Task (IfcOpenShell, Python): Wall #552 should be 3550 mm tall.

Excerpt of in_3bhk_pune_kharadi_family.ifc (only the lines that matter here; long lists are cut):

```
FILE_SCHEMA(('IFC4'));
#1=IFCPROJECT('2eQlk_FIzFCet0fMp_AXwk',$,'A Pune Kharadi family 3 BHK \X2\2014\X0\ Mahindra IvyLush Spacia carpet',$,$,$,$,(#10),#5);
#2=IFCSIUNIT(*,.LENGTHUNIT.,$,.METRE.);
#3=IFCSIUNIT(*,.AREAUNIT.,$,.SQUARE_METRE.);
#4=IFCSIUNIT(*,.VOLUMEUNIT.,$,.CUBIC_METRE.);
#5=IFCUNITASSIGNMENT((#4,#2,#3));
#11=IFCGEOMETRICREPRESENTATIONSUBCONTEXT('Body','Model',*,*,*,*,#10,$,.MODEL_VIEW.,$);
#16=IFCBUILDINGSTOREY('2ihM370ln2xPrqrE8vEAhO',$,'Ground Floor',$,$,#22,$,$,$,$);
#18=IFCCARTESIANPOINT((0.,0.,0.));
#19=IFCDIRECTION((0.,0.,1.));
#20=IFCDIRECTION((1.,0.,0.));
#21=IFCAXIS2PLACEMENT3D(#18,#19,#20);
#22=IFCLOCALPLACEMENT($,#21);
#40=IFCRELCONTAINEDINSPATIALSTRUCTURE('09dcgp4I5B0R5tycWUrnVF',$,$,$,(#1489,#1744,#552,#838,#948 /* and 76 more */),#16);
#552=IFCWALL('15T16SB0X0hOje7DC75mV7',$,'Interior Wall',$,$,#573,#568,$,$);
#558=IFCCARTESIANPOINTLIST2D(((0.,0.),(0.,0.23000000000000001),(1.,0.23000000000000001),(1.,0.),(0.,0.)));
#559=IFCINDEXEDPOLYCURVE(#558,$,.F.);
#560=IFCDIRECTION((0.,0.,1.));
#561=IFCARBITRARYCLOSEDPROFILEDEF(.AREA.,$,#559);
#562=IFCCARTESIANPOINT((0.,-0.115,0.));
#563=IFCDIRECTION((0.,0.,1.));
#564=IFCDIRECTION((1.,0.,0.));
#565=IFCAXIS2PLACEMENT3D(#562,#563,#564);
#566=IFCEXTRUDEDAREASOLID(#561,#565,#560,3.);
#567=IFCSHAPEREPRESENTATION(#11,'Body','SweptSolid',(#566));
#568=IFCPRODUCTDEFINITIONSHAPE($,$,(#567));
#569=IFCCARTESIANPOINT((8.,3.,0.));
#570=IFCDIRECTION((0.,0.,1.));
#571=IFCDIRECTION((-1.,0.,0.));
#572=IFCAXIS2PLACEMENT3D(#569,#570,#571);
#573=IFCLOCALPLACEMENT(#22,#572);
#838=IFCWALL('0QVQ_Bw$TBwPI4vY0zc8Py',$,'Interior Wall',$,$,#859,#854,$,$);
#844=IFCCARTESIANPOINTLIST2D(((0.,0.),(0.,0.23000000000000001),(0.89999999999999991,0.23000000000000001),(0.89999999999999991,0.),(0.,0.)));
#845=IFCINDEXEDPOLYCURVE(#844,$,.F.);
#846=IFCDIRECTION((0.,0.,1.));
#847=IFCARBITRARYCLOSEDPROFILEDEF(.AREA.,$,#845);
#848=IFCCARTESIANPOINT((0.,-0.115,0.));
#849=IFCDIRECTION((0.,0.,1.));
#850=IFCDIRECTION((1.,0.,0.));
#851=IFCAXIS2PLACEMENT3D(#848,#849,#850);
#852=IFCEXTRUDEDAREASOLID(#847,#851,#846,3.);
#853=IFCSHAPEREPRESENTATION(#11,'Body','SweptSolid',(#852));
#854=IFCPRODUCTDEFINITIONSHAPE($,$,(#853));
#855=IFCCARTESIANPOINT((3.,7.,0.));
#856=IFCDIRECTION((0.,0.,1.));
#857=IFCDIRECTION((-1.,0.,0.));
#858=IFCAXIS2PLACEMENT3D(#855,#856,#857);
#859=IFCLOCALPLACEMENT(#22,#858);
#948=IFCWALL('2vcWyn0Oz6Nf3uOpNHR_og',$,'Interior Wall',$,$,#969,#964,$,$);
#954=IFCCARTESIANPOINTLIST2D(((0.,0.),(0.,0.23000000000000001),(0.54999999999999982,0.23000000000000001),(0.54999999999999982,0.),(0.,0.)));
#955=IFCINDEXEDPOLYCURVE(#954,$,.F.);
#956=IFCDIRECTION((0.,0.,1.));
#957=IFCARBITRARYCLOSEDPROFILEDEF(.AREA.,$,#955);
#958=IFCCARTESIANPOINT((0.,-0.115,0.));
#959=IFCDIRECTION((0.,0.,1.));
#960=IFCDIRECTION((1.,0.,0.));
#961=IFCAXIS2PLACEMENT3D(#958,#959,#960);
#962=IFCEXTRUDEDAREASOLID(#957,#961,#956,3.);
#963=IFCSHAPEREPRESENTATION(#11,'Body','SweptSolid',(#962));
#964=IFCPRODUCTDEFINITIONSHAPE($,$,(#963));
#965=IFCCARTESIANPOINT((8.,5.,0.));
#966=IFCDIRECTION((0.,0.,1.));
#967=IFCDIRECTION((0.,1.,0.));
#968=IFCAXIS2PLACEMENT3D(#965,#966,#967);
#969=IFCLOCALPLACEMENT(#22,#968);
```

```python
import ifcopenshell
import ifcopenshell.geom
import ifcopenshell.util.representation
import ifcopenshell.util.shape

model = ifcopenshell.open("in_3bhk_pune_kharadi_family.ifc")
settings = ifcopenshell.geom.settings()


def volume(element):
    """Net volume in cubic metres, openings subtracted."""
    shape = ifcopenshell.geom.create_shape(settings, element)
    return ifcopenshell.util.shape.get_volume(shape.geometry)


wall = model.by_guid("15T16SB0X0hOje7DC75mV7")
before = volume(wall)

body = ifcopenshell.util.representation.get_representation(wall, "Model", "Body")
solid = body.Items[0]
old_height = solid.Depth
solid.Depth = 3.55
after = volume(wall)

print(f"height {old_height:g} -> {solid.Depth:g}, volume {before:.3f} -> {after:.3f} m3")

model.write("in_3bhk_pune_kharadi_family_updated.ifc")
```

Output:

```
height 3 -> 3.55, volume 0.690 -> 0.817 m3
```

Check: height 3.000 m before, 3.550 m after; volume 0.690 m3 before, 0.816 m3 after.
